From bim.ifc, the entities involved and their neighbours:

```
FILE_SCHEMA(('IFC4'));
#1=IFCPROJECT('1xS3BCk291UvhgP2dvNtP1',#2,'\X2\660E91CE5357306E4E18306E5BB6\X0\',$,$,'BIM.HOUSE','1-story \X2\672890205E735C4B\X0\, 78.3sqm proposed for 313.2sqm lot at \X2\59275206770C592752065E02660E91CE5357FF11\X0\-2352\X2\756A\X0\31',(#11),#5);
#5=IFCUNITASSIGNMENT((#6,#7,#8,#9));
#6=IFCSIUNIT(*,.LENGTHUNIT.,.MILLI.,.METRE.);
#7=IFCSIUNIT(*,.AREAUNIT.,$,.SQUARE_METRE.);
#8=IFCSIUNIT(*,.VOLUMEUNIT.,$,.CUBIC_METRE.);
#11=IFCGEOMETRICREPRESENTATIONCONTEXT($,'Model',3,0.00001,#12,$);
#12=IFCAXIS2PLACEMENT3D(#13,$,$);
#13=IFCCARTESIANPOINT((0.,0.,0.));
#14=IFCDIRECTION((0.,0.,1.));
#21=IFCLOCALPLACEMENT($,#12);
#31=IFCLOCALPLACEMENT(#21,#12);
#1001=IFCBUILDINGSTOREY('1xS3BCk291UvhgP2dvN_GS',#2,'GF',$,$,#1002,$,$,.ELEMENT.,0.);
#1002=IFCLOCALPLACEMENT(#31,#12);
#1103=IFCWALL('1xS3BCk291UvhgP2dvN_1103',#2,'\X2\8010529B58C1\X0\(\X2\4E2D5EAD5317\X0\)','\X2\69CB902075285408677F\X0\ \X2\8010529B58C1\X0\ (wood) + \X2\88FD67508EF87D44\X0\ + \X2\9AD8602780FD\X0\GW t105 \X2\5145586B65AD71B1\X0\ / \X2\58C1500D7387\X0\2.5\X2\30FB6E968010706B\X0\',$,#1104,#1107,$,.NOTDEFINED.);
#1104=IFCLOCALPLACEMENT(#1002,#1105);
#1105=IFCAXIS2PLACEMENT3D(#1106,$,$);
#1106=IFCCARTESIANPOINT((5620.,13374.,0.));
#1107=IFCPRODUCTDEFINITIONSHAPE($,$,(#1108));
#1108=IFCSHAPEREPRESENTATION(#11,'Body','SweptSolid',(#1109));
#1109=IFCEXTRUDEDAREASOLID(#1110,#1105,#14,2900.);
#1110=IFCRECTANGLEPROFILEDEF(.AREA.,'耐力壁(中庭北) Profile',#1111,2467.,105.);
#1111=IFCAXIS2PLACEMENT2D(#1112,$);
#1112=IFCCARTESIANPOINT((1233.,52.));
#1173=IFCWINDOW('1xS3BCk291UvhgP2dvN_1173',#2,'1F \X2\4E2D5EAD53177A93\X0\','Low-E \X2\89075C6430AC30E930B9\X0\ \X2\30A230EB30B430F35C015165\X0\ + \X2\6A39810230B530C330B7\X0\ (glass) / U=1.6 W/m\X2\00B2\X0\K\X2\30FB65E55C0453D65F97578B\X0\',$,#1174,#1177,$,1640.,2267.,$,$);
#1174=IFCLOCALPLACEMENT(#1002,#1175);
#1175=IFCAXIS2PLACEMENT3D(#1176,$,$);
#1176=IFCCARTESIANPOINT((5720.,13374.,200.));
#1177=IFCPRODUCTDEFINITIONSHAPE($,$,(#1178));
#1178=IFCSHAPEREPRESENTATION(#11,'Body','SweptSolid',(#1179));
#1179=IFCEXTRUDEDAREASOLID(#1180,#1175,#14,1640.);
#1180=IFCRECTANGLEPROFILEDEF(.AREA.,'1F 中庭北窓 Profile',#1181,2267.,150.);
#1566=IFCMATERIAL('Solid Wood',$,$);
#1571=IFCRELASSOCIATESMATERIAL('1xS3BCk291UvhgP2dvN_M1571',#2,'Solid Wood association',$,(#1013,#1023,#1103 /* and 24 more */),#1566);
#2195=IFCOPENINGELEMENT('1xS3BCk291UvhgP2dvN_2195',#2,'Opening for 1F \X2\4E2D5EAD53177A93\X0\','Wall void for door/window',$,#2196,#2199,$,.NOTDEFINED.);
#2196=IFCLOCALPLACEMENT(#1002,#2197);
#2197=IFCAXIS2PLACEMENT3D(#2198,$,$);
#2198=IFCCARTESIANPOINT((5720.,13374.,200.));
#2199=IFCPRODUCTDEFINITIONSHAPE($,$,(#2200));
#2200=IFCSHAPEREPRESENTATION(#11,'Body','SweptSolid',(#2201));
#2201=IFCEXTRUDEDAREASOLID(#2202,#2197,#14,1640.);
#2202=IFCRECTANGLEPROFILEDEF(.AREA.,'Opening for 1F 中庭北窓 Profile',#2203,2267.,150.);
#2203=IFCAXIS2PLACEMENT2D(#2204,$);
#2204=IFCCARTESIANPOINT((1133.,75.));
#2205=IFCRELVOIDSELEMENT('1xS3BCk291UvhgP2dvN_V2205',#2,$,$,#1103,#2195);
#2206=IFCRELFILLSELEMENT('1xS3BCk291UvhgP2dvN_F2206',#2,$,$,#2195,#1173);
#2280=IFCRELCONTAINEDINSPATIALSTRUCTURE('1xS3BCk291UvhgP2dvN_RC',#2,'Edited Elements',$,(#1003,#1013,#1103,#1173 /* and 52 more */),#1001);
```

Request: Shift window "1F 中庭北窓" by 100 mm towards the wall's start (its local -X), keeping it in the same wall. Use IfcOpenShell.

```python
import ifcopenshell
import ifcopenshell.api.geometry
import ifcopenshell.util.placement
import ifcopenshell.util.unit

model = ifcopenshell.open("bim.ifc")
unit_scale = ifcopenshell.util.unit.calculate_unit_scale(model)

window = model.by_guid("1xS3BCk291UvhgP2dvN_1173")
opening = window.FillsVoids[0].RelatingOpeningElement
wall = opening.VoidsElements[0].RelatingBuildingElement

wall_matrix = ifcopenshell.util.placement.get_local_placement(wall.ObjectPlacement)
shift = wall_matrix[:3, 0] * -0.1 / unit_scale
before = ifcopenshell.util.placement.get_local_placement(window.ObjectPlacement)[:3, 3].copy()

# The window is not placed relative to its opening, so move both.
for product in (opening, window):
    matrix = ifcopenshell.util.placement.get_local_placement(product.ObjectPlacement)
    matrix[:3, 3] += shift
    ifcopenshell.api.geometry.edit_object_placement(model, product=product, matrix=matrix, is_si=False)

after = ifcopenshell.util.placement.get_local_placement(window.ObjectPlacement)[:3, 3]
print("window moved by", (after - before).round(3) + 0.0)

model.write("bim-out.ifc")
```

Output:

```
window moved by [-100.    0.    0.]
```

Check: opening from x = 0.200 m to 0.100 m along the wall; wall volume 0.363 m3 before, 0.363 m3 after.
